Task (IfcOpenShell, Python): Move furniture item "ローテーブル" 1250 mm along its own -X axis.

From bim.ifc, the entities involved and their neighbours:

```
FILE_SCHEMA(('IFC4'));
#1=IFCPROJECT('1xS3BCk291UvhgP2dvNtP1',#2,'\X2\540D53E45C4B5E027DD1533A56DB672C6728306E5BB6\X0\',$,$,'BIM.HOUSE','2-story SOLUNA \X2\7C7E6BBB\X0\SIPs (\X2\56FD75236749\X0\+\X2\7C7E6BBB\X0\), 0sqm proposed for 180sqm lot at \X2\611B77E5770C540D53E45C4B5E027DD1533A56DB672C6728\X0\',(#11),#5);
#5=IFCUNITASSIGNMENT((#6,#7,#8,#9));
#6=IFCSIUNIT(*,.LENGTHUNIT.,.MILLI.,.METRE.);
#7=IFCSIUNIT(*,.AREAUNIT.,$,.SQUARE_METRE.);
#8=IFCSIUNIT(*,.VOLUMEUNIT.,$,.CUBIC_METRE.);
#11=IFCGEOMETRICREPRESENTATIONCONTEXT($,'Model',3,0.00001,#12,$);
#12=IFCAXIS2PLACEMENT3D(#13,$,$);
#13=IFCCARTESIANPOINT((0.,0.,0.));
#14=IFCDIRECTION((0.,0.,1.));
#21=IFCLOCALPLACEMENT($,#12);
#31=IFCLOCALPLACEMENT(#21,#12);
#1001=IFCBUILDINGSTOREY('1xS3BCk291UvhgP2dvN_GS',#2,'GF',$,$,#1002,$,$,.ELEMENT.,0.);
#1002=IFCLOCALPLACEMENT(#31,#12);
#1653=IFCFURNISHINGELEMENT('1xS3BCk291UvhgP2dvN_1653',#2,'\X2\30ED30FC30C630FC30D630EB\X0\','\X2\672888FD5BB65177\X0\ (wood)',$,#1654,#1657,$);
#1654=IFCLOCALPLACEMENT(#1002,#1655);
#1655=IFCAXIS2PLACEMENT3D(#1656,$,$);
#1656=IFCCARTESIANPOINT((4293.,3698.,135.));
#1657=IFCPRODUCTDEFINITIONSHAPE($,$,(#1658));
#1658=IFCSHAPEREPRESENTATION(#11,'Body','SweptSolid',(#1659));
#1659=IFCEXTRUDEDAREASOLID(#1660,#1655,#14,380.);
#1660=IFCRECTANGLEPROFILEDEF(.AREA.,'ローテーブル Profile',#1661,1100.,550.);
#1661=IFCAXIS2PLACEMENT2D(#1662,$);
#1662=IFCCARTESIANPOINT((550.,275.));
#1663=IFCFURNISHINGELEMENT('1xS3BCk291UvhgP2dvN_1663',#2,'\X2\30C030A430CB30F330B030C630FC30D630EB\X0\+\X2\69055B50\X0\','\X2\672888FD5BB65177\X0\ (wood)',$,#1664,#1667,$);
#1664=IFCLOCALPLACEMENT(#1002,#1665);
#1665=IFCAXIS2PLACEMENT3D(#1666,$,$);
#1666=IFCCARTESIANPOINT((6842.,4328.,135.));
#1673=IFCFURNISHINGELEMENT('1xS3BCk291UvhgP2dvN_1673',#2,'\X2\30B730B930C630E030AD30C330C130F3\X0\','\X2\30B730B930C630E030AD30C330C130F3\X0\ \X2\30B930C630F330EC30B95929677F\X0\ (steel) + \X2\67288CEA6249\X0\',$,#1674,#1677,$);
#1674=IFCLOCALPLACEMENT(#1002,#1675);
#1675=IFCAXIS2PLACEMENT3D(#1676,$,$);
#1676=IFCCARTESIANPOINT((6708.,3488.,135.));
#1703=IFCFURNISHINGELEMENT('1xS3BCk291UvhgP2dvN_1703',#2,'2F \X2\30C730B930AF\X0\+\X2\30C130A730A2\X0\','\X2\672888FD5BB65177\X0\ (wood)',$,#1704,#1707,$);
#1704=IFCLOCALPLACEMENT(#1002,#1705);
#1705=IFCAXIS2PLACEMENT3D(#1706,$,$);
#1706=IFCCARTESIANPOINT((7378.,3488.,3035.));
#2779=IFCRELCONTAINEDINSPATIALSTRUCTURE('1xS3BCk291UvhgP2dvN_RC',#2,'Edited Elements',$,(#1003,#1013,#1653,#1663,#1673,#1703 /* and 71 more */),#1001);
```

```python
import ifcopenshell
import ifcopenshell.api.geometry
import ifcopenshell.util.placement

model = ifcopenshell.open("bim.ifc")

item = model.by_id(1653)
matrix = ifcopenshell.util.placement.get_local_placement(item.ObjectPlacement)
matrix[:3, 3] -= matrix[:3, 0] * 1250.0
ifcopenshell.api.geometry.edit_object_placement(model, product=item, matrix=matrix, is_si=False)

print(ifcopenshell.util.placement.get_local_placement(item.ObjectPlacement).round(3) + 0.0)

model.write("bim_updated.ifc")
```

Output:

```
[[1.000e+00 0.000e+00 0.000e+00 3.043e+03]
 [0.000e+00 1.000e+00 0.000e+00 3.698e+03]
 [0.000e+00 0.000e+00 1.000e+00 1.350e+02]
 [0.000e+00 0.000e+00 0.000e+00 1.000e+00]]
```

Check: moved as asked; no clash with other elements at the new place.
